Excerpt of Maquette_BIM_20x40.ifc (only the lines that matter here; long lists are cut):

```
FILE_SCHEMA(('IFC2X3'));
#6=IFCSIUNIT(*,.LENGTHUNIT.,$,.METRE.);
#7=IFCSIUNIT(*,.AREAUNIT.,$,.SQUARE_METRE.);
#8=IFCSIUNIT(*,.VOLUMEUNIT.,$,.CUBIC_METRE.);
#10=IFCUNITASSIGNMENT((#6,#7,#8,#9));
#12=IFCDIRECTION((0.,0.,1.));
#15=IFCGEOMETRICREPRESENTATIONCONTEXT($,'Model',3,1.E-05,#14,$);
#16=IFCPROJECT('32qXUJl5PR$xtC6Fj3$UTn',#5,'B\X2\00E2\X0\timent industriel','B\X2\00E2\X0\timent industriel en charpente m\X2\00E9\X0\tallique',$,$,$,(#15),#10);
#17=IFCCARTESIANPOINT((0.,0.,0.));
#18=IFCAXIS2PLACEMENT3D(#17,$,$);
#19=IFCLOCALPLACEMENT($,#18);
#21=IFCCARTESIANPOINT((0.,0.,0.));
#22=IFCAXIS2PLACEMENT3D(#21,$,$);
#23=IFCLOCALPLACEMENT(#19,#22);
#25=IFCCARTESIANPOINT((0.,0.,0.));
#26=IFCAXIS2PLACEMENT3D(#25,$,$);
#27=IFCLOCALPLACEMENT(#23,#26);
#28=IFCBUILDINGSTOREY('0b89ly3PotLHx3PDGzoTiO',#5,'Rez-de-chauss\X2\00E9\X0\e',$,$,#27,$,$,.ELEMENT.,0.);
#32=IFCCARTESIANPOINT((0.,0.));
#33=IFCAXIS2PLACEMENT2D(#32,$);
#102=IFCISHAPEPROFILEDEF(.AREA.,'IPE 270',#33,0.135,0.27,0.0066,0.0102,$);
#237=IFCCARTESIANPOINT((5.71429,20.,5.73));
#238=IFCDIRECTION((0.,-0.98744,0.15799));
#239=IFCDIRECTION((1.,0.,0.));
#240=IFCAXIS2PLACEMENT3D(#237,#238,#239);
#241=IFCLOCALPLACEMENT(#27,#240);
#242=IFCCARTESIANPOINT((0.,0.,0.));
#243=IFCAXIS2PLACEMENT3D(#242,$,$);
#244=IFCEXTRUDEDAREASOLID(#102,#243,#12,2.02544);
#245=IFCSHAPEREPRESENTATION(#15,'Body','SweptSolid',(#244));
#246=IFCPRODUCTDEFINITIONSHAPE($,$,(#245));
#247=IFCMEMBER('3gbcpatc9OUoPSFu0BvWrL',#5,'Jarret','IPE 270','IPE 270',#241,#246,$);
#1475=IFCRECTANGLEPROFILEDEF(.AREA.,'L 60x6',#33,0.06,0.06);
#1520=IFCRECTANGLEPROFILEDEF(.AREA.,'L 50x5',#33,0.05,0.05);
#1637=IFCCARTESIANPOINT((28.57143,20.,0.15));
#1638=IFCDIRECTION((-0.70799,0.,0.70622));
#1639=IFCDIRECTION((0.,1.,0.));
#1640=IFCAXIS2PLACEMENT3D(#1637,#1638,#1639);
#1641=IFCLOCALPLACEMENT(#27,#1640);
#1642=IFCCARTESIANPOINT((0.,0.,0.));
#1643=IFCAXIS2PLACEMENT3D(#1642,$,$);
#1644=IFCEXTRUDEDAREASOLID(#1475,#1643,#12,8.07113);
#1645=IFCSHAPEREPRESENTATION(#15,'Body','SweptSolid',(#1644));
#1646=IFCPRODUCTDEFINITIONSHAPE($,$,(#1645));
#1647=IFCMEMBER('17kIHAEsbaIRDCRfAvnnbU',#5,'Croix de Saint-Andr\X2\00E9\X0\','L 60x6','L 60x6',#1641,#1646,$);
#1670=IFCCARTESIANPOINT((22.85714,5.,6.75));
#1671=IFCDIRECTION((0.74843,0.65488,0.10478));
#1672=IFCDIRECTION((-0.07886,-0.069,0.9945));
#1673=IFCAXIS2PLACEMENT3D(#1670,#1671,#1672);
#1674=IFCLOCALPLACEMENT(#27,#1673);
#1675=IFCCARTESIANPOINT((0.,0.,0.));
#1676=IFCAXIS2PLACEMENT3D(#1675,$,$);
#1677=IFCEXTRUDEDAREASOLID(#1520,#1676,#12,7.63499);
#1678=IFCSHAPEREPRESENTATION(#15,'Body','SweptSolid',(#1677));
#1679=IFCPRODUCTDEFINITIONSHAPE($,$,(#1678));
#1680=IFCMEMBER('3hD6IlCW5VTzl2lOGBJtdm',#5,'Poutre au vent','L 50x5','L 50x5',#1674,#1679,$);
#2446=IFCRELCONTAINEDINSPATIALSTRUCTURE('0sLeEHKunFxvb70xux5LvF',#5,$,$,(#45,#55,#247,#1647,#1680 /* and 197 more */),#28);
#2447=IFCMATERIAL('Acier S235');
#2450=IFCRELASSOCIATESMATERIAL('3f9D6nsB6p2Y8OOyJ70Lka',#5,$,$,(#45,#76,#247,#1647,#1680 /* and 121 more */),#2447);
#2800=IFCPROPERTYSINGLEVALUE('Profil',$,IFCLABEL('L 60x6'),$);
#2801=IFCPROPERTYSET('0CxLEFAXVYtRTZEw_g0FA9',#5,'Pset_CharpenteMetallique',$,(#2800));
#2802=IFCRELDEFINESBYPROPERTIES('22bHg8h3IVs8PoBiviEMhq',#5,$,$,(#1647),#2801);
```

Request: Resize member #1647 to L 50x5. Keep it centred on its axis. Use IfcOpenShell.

```python
import ifcopenshell
import ifcopenshell.api.pset
import ifcopenshell.util.element

model = ifcopenshell.open("Maquette_BIM_20x40.ifc")

member = model.by_id(1647)
source = next(p for p in model.by_type("IfcRectangleProfileDef") if p.ProfileName == "L 50x5")

body = next(r for r in member.Representation.Representations if r.RepresentationIdentifier == "Body")
solid = body.Items[0]
old_profile = solid.SweptArea

# Copy the section's sizes but keep this member's own profile position.
profile = ifcopenshell.util.element.copy(model, source)
profile.Position = old_profile.Position
solid.SweptArea = profile
if not model.get_total_inverses(old_profile):
    ifcopenshell.util.element.remove_deep2(model, old_profile)
member.Description = member.Description.replace("L 60x6", "L 50x5")
member.ObjectType = member.ObjectType.replace("L 60x6", "L 50x5")
pset = model.by_id(ifcopenshell.util.element.get_pset(member, "Pset_CharpenteMetallique", should_inherit=False)["id"])
ifcopenshell.api.pset.edit_pset(model, pset=pset, properties={"Profil": "L 50x5"})

print(solid.SweptArea)

model.write("Maquette_BIM_20x40_rev.ifc")
```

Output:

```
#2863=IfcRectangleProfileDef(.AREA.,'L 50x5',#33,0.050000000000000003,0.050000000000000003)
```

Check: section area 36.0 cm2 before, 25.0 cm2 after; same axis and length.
